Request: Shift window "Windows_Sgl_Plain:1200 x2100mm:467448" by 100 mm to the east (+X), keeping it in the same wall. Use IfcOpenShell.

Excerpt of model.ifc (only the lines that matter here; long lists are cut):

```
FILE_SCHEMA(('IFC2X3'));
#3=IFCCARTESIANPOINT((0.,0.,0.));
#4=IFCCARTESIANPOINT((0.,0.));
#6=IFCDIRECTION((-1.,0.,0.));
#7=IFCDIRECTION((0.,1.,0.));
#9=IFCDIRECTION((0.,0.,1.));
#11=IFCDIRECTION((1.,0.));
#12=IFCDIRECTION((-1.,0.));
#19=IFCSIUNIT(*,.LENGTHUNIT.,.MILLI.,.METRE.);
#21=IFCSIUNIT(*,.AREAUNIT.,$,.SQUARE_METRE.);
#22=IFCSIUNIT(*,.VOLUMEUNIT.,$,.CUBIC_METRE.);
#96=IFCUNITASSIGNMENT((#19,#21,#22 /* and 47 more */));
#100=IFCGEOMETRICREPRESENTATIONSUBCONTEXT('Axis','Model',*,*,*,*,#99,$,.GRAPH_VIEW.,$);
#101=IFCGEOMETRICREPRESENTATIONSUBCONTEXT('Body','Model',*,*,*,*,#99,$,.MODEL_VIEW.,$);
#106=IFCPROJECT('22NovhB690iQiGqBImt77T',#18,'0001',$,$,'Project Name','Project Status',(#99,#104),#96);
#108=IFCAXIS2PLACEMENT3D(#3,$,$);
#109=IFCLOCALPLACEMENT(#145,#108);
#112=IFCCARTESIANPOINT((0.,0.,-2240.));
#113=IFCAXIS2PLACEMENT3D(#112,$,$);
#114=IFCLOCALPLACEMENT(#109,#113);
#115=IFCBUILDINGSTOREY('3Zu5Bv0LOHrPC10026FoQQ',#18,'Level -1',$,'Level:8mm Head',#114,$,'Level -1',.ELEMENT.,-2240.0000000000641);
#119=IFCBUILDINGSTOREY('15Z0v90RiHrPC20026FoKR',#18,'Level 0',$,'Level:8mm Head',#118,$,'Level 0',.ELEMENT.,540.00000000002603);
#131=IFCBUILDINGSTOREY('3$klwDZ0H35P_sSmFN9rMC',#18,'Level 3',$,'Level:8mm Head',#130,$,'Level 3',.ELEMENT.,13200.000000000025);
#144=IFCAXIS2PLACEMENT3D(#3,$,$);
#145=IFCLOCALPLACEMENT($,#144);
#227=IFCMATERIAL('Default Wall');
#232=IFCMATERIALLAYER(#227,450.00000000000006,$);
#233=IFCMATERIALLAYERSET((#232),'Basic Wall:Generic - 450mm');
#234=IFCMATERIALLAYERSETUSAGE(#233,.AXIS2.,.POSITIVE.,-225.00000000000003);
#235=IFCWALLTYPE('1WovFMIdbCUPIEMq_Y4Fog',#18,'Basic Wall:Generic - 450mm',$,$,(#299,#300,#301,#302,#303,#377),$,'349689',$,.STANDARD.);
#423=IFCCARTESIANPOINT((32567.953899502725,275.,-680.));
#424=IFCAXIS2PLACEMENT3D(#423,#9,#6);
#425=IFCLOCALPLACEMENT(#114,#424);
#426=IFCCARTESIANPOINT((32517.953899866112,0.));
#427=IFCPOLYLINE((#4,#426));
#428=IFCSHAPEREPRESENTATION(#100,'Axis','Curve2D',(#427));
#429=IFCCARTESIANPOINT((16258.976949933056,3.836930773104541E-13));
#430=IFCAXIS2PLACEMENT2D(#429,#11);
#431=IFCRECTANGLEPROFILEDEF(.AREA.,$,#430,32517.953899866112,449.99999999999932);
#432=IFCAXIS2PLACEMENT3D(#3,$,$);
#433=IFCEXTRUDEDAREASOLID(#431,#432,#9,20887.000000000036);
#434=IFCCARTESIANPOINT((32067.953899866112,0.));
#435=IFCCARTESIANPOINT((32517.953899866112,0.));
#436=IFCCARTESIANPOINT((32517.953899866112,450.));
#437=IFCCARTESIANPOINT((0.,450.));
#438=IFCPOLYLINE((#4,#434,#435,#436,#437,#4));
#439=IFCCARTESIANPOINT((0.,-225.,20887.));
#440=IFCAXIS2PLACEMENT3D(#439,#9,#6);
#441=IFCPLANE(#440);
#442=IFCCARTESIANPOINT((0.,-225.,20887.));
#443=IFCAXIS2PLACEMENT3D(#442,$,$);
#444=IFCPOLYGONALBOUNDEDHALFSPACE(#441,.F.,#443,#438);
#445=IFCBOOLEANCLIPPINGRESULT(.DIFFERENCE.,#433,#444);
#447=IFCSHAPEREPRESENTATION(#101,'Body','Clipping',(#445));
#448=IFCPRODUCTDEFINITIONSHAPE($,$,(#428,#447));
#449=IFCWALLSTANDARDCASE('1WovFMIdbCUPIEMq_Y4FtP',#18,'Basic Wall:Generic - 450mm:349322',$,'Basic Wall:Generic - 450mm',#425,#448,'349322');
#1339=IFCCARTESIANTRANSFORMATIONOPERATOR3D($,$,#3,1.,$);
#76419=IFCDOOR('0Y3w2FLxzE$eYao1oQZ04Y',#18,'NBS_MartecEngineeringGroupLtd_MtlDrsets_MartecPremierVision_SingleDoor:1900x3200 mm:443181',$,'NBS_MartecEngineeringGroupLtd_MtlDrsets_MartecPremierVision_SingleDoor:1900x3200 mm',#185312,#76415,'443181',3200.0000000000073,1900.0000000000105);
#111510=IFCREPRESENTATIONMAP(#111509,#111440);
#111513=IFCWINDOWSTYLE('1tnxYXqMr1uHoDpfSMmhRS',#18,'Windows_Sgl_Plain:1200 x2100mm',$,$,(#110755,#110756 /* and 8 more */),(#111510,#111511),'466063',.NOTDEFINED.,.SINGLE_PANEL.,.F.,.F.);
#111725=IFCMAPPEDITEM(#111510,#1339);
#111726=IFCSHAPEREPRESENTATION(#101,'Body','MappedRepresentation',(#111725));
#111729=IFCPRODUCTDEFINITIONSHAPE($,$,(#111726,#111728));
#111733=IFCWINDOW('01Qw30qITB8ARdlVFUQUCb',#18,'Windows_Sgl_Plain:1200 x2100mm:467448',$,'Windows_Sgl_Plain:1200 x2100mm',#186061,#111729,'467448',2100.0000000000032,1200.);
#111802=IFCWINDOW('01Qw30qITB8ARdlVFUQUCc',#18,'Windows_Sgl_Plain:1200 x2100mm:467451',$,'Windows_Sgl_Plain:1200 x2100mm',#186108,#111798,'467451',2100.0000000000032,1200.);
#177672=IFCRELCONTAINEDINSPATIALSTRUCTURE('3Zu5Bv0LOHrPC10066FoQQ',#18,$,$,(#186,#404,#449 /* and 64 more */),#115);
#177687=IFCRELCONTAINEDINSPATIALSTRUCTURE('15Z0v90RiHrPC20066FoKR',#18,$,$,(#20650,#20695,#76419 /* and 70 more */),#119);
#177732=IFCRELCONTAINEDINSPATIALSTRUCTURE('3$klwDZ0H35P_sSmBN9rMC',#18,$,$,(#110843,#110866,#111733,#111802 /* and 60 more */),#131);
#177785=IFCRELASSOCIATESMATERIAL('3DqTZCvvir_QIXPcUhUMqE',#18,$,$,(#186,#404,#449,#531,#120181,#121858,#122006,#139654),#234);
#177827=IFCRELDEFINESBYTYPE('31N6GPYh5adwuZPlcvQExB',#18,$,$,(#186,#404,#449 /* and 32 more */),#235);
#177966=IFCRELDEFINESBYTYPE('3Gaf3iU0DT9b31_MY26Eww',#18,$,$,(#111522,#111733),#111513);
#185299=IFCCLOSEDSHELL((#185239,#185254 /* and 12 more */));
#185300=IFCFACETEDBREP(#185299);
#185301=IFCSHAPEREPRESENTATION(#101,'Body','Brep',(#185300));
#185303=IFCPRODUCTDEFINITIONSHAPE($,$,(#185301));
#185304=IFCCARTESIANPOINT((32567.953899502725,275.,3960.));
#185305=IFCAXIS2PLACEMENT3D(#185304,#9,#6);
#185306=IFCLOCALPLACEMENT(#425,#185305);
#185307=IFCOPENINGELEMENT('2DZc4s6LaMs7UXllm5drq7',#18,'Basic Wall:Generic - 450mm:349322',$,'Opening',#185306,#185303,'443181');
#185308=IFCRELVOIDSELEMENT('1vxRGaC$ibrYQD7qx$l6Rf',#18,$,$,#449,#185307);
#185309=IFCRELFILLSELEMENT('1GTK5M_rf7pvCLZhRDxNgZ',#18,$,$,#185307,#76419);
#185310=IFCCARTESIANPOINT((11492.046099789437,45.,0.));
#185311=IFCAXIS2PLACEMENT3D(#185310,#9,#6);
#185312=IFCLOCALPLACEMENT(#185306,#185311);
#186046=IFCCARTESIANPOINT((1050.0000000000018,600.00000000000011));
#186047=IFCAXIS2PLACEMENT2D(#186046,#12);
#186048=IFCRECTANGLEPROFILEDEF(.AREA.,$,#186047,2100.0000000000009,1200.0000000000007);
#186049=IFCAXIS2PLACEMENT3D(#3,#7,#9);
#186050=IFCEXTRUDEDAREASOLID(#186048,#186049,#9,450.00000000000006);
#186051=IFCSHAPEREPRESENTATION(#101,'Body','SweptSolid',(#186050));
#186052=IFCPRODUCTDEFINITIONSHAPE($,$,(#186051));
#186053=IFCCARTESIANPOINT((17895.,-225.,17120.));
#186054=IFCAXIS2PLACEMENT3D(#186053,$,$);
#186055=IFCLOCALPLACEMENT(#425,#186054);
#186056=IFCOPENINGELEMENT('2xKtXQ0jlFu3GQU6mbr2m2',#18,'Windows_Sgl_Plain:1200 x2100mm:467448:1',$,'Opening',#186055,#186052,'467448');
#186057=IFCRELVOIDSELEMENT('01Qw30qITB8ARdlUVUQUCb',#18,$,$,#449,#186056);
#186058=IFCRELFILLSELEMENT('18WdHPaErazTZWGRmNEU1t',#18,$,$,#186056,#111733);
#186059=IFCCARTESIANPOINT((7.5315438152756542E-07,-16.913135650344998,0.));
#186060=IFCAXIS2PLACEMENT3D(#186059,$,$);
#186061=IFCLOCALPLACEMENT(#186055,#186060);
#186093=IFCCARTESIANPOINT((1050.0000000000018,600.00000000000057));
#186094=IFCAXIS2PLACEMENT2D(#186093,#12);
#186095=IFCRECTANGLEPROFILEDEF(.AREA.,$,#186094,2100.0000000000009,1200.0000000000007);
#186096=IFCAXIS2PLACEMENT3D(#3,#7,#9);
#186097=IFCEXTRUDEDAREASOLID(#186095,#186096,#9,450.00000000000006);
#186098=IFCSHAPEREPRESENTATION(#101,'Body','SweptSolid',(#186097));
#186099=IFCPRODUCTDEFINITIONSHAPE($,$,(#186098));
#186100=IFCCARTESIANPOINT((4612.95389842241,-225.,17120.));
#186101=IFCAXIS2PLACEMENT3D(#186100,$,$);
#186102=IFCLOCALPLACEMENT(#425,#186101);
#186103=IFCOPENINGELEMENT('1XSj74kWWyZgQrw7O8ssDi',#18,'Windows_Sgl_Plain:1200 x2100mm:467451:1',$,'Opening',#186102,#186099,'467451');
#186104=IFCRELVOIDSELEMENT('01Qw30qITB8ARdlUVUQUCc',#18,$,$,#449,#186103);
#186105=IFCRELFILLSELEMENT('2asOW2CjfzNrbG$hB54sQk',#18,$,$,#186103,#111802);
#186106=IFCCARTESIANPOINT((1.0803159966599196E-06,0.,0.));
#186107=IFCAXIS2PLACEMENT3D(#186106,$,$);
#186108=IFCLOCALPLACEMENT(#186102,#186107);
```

```python
import ifcopenshell
import ifcopenshell.api.geometry
import ifcopenshell.util.placement
import ifcopenshell.util.unit

model = ifcopenshell.open("model.ifc")
unit_scale = ifcopenshell.util.unit.calculate_unit_scale(model)

window = model.by_id(111733)
opening = window.FillsVoids[0].RelatingOpeningElement
wall = opening.VoidsElements[0].RelatingBuildingElement

wall_matrix = ifcopenshell.util.placement.get_local_placement(wall.ObjectPlacement)
shift = wall_matrix[:3, 0] * -0.1 / unit_scale
before = ifcopenshell.util.placement.get_local_placement(window.ObjectPlacement)[:3, 3].copy()

# The window is placed relative to its opening, so it follows when the opening moves.
matrix = ifcopenshell.util.placement.get_local_placement(opening.ObjectPlacement)
matrix[:3, 3] += shift
ifcopenshell.api.geometry.edit_object_placement(
    model, product=opening, matrix=matrix, is_si=False, should_transform_children=True
)

after = ifcopenshell.util.placement.get_local_placement(window.ObjectPlacement)[:3, 3]
print("window moved by", (after - before).round(3) + 0.0)

model.write("model_edited.ifc")
```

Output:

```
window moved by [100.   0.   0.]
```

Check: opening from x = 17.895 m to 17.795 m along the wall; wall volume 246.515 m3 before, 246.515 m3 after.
